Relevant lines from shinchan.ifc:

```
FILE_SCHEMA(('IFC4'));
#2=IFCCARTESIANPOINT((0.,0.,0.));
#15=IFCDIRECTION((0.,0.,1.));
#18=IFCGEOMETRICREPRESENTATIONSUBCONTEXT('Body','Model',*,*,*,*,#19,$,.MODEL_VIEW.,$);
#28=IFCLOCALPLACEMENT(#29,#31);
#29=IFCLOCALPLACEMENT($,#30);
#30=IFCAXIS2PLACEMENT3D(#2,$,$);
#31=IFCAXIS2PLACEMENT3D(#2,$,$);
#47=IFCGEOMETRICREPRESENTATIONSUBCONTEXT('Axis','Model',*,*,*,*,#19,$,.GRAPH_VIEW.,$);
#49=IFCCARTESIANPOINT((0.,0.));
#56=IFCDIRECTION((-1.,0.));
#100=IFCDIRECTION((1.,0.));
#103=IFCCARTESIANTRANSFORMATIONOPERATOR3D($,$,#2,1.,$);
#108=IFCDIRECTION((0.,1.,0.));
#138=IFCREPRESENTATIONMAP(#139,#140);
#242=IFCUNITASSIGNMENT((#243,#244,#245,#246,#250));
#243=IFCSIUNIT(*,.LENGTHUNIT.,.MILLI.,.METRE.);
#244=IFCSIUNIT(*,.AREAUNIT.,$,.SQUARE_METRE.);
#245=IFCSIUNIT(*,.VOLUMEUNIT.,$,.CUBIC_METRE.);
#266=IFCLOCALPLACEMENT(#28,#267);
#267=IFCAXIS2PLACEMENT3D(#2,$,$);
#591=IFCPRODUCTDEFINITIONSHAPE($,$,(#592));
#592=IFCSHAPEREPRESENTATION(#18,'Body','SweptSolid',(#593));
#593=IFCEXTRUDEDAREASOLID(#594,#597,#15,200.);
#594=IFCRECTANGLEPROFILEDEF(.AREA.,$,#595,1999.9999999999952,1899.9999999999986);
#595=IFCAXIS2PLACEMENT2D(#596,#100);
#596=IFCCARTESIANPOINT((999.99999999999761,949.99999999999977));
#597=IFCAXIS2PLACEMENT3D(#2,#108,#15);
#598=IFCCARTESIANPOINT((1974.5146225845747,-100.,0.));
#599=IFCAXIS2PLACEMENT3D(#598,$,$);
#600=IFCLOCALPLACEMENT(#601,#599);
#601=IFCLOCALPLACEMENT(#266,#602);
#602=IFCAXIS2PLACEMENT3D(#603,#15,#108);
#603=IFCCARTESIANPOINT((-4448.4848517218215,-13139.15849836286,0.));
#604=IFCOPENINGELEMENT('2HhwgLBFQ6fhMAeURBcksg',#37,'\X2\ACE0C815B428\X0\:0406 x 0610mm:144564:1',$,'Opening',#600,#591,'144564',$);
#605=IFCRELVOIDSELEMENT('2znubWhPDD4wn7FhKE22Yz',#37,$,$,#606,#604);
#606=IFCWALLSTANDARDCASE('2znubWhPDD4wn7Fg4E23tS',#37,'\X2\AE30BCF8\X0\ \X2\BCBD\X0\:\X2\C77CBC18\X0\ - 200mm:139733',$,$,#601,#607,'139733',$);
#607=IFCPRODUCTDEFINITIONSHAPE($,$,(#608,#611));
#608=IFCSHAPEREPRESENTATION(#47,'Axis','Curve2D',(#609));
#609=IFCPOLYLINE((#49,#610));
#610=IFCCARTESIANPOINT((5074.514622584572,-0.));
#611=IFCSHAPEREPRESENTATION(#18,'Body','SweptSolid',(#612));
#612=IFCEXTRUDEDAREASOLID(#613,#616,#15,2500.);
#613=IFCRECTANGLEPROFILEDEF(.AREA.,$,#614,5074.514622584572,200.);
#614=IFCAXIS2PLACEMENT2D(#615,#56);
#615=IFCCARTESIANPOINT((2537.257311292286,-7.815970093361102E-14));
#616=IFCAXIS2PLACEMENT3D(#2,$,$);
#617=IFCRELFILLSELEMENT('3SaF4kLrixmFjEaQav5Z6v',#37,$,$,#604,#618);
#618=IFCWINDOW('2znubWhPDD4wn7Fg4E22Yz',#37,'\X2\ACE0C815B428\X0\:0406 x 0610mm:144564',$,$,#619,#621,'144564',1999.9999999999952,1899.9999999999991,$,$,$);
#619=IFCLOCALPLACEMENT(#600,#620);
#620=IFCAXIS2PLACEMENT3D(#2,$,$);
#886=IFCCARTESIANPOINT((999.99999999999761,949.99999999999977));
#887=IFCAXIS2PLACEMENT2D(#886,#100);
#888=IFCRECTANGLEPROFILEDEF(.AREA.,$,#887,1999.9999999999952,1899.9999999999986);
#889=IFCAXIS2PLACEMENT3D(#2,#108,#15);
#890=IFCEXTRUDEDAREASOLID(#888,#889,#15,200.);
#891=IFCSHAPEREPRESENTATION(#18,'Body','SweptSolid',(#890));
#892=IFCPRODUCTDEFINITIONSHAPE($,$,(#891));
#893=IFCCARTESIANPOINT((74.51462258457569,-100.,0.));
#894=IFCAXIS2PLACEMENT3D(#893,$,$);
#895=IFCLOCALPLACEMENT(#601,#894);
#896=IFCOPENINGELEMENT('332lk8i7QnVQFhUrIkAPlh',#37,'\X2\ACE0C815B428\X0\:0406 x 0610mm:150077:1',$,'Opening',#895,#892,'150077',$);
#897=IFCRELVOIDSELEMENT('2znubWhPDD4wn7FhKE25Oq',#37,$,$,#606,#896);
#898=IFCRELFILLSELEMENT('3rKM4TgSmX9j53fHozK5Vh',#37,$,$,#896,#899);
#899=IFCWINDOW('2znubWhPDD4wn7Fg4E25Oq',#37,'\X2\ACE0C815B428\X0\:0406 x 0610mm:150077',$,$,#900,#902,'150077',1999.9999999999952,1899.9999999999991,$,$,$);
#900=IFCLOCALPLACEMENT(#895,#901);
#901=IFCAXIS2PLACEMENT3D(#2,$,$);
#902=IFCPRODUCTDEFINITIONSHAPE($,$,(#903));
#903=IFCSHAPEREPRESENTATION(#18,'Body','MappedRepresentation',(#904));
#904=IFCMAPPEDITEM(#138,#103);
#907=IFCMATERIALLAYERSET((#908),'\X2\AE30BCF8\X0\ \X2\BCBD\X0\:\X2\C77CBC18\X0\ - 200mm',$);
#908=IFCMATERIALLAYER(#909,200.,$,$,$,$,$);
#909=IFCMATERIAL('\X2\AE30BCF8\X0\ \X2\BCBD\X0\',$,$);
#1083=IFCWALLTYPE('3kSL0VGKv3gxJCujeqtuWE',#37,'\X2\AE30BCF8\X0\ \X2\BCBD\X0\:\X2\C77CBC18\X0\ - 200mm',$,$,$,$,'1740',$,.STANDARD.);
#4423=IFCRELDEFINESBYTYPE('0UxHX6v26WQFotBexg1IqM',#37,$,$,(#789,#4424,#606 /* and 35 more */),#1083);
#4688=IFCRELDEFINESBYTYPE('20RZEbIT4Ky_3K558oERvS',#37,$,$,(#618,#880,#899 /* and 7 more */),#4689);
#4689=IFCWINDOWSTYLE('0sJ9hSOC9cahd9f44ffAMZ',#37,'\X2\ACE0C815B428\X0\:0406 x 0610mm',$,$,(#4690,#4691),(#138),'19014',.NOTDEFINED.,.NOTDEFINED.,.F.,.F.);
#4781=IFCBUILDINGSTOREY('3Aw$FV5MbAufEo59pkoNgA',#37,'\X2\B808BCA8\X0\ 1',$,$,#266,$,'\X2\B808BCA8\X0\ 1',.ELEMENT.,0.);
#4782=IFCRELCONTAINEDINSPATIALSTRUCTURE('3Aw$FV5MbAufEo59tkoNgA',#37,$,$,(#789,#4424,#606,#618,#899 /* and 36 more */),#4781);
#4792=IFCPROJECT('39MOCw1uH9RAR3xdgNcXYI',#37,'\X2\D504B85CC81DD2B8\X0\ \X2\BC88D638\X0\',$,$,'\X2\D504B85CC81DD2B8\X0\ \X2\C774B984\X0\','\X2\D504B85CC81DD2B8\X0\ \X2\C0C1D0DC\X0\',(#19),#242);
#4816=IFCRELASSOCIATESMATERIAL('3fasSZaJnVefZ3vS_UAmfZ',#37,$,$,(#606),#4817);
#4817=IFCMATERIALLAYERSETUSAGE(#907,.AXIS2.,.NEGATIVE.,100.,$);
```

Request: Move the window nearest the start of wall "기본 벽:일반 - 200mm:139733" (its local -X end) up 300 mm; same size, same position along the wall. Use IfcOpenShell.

```python
import numpy as np
import ifcopenshell
import ifcopenshell.api.geometry
import ifcopenshell.util.placement
import ifcopenshell.util.unit

model = ifcopenshell.open("shinchan.ifc")
unit_scale = ifcopenshell.util.unit.calculate_unit_scale(model)

window = model.by_id(899)
opening = window.FillsVoids[0].RelatingOpeningElement
dz = 0.3 / unit_scale

shift = np.array([0.0, 0.0, dz])
# The window is placed relative to its opening, so it follows when the opening moves.
matrix = ifcopenshell.util.placement.get_local_placement(opening.ObjectPlacement)
matrix[:3, 3] += shift
ifcopenshell.api.geometry.edit_object_placement(
    model, product=opening, matrix=matrix, is_si=False, should_transform_children=True
)

print(f"moved by {dz * unit_scale:+.3f} m")

model.write("shinchan_edited.ifc")
```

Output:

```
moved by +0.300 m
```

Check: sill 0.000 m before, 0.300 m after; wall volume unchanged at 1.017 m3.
